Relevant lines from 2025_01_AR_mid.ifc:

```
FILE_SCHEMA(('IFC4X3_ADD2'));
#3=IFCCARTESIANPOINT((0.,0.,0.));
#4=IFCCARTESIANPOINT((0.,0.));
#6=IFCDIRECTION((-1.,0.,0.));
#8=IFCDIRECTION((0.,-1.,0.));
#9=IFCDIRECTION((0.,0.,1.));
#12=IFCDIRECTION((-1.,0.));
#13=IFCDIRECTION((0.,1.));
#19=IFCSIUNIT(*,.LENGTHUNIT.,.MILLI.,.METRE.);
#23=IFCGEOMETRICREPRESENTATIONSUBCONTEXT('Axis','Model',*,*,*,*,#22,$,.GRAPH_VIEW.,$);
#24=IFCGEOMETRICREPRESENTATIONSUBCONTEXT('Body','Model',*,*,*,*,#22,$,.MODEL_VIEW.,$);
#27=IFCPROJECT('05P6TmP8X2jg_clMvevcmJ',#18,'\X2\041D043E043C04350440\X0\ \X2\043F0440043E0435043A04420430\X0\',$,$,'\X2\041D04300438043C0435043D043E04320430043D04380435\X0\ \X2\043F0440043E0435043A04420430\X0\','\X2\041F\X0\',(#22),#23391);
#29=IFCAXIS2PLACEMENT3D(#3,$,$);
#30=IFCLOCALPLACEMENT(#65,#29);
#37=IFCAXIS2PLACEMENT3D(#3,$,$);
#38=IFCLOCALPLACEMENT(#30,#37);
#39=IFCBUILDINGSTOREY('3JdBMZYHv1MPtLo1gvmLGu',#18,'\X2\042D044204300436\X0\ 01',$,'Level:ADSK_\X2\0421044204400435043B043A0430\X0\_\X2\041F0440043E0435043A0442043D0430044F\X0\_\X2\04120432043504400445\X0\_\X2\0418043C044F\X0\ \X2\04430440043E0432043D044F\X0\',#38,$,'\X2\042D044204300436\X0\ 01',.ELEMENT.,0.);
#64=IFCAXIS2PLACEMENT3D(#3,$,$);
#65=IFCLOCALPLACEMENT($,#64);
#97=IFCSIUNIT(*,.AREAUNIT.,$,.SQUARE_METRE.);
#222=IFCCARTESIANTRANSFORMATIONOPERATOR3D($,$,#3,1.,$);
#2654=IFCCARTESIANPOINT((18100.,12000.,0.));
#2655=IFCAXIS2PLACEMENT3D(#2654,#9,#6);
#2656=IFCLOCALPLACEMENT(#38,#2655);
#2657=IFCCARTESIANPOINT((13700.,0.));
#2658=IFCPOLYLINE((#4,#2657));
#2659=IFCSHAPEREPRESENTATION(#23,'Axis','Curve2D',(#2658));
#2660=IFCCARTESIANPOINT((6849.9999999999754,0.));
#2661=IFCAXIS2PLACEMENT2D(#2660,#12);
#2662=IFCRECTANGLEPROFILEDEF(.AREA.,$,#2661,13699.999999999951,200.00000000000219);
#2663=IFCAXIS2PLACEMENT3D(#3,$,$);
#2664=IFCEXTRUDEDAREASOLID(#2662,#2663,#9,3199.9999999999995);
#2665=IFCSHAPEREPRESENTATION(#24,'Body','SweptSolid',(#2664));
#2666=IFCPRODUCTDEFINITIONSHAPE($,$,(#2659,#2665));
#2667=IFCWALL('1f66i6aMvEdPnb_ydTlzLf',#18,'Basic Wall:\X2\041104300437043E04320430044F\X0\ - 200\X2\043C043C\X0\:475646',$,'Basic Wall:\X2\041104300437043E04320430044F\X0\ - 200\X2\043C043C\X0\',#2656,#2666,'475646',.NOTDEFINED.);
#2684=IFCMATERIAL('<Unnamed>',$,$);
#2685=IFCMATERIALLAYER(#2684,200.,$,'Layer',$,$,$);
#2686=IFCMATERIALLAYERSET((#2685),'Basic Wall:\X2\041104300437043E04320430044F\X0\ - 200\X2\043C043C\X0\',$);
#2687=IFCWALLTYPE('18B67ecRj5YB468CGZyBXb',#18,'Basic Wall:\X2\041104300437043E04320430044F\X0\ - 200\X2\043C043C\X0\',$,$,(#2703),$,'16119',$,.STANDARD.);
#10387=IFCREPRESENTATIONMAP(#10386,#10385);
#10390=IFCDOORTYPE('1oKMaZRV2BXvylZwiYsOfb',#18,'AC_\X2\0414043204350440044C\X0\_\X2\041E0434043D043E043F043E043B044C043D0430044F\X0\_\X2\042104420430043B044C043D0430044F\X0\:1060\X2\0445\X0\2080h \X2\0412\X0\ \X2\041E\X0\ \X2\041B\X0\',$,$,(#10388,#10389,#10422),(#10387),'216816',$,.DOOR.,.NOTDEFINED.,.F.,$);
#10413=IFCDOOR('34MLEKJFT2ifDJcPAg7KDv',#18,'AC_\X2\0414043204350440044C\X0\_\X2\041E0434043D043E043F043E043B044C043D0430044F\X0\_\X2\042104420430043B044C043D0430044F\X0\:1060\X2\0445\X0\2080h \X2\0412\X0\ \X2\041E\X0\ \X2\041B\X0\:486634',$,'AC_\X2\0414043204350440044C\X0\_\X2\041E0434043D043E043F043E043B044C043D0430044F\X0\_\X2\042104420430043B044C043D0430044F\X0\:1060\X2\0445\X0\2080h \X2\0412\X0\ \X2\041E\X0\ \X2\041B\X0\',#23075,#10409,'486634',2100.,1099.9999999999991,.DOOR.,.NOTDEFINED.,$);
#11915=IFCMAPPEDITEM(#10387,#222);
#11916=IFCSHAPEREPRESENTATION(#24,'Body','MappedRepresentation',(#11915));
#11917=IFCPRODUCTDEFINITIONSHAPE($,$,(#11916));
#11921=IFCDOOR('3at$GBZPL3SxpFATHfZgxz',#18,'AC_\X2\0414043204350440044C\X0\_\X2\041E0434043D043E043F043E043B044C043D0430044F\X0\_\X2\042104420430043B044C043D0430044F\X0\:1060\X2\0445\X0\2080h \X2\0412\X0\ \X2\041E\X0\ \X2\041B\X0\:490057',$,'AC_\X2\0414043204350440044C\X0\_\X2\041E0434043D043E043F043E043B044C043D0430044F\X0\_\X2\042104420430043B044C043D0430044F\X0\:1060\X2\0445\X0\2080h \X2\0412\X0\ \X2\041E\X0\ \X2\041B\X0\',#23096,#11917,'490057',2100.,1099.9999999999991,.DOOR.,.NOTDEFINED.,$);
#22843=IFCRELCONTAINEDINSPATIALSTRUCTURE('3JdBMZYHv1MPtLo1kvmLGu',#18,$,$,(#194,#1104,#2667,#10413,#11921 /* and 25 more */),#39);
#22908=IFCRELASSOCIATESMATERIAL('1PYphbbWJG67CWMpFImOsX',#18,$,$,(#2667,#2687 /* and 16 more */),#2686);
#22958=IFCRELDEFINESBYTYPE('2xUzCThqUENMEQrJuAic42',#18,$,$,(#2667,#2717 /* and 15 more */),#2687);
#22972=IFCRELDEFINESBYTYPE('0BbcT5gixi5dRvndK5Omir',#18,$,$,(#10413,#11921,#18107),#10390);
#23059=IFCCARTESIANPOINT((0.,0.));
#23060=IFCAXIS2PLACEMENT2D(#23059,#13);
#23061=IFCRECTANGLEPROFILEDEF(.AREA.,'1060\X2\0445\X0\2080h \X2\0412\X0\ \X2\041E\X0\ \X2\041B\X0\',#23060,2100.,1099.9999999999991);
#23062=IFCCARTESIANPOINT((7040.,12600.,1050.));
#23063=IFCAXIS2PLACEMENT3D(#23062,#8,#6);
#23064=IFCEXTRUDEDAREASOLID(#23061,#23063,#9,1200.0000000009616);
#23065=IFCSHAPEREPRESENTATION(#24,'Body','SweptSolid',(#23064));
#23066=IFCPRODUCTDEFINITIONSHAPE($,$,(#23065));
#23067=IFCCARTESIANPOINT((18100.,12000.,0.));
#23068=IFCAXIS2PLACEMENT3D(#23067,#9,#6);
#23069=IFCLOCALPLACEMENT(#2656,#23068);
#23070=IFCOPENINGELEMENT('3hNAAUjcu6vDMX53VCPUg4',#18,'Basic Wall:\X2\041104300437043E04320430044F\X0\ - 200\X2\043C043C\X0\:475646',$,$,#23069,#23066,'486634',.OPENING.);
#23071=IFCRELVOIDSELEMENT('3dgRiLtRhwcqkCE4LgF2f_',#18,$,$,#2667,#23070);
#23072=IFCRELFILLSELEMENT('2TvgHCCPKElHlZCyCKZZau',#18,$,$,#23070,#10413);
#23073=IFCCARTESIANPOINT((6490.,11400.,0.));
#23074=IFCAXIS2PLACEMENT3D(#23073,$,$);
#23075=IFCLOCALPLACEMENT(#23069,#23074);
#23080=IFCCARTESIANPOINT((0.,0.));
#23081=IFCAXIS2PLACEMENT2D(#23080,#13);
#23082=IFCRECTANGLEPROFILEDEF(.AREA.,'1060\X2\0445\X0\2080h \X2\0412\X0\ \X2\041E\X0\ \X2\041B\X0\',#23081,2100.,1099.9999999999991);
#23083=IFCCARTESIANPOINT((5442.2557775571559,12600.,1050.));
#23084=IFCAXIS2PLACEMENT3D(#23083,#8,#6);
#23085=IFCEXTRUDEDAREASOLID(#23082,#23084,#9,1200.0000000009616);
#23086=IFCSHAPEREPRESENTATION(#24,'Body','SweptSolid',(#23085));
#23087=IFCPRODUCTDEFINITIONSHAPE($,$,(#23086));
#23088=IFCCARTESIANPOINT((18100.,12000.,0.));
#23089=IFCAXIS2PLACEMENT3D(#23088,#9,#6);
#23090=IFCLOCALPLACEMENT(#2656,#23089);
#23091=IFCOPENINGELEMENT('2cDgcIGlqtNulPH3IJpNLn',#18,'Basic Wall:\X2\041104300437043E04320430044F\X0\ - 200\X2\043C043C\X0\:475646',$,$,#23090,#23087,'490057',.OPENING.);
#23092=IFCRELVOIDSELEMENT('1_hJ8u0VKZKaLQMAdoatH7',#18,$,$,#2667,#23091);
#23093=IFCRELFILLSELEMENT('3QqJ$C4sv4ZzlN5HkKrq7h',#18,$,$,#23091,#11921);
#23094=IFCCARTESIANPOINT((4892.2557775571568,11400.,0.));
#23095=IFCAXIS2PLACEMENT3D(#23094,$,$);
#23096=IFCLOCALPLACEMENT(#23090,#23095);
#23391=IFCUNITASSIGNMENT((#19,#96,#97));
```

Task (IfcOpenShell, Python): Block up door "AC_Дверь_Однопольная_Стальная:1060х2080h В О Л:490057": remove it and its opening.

```python
import ifcopenshell
import ifcopenshell.api.feature
import ifcopenshell.api.root
import ifcopenshell.geom
import ifcopenshell.util.shape

model = ifcopenshell.open("2025_01_AR_mid.ifc")
settings = ifcopenshell.geom.settings()


def volume(element):
    """Net volume in cubic metres, openings subtracted."""
    shape = ifcopenshell.geom.create_shape(settings, element)
    return ifcopenshell.util.shape.get_volume(shape.geometry)


door = model.by_id(11921)
opening = door.FillsVoids[0].RelatingOpeningElement
wall = opening.VoidsElements[0].RelatingBuildingElement
before = volume(wall)

ifcopenshell.api.root.remove_product(model, product=door)
ifcopenshell.api.feature.remove_feature(model, feature=opening)

after = volume(wall)

print(f"wall volume {before:.3f} -> {after:.3f} m3")

model.write("2025_01_AR_mid_updated.ifc")
```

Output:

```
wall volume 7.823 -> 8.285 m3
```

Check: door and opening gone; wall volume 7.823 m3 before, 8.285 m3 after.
